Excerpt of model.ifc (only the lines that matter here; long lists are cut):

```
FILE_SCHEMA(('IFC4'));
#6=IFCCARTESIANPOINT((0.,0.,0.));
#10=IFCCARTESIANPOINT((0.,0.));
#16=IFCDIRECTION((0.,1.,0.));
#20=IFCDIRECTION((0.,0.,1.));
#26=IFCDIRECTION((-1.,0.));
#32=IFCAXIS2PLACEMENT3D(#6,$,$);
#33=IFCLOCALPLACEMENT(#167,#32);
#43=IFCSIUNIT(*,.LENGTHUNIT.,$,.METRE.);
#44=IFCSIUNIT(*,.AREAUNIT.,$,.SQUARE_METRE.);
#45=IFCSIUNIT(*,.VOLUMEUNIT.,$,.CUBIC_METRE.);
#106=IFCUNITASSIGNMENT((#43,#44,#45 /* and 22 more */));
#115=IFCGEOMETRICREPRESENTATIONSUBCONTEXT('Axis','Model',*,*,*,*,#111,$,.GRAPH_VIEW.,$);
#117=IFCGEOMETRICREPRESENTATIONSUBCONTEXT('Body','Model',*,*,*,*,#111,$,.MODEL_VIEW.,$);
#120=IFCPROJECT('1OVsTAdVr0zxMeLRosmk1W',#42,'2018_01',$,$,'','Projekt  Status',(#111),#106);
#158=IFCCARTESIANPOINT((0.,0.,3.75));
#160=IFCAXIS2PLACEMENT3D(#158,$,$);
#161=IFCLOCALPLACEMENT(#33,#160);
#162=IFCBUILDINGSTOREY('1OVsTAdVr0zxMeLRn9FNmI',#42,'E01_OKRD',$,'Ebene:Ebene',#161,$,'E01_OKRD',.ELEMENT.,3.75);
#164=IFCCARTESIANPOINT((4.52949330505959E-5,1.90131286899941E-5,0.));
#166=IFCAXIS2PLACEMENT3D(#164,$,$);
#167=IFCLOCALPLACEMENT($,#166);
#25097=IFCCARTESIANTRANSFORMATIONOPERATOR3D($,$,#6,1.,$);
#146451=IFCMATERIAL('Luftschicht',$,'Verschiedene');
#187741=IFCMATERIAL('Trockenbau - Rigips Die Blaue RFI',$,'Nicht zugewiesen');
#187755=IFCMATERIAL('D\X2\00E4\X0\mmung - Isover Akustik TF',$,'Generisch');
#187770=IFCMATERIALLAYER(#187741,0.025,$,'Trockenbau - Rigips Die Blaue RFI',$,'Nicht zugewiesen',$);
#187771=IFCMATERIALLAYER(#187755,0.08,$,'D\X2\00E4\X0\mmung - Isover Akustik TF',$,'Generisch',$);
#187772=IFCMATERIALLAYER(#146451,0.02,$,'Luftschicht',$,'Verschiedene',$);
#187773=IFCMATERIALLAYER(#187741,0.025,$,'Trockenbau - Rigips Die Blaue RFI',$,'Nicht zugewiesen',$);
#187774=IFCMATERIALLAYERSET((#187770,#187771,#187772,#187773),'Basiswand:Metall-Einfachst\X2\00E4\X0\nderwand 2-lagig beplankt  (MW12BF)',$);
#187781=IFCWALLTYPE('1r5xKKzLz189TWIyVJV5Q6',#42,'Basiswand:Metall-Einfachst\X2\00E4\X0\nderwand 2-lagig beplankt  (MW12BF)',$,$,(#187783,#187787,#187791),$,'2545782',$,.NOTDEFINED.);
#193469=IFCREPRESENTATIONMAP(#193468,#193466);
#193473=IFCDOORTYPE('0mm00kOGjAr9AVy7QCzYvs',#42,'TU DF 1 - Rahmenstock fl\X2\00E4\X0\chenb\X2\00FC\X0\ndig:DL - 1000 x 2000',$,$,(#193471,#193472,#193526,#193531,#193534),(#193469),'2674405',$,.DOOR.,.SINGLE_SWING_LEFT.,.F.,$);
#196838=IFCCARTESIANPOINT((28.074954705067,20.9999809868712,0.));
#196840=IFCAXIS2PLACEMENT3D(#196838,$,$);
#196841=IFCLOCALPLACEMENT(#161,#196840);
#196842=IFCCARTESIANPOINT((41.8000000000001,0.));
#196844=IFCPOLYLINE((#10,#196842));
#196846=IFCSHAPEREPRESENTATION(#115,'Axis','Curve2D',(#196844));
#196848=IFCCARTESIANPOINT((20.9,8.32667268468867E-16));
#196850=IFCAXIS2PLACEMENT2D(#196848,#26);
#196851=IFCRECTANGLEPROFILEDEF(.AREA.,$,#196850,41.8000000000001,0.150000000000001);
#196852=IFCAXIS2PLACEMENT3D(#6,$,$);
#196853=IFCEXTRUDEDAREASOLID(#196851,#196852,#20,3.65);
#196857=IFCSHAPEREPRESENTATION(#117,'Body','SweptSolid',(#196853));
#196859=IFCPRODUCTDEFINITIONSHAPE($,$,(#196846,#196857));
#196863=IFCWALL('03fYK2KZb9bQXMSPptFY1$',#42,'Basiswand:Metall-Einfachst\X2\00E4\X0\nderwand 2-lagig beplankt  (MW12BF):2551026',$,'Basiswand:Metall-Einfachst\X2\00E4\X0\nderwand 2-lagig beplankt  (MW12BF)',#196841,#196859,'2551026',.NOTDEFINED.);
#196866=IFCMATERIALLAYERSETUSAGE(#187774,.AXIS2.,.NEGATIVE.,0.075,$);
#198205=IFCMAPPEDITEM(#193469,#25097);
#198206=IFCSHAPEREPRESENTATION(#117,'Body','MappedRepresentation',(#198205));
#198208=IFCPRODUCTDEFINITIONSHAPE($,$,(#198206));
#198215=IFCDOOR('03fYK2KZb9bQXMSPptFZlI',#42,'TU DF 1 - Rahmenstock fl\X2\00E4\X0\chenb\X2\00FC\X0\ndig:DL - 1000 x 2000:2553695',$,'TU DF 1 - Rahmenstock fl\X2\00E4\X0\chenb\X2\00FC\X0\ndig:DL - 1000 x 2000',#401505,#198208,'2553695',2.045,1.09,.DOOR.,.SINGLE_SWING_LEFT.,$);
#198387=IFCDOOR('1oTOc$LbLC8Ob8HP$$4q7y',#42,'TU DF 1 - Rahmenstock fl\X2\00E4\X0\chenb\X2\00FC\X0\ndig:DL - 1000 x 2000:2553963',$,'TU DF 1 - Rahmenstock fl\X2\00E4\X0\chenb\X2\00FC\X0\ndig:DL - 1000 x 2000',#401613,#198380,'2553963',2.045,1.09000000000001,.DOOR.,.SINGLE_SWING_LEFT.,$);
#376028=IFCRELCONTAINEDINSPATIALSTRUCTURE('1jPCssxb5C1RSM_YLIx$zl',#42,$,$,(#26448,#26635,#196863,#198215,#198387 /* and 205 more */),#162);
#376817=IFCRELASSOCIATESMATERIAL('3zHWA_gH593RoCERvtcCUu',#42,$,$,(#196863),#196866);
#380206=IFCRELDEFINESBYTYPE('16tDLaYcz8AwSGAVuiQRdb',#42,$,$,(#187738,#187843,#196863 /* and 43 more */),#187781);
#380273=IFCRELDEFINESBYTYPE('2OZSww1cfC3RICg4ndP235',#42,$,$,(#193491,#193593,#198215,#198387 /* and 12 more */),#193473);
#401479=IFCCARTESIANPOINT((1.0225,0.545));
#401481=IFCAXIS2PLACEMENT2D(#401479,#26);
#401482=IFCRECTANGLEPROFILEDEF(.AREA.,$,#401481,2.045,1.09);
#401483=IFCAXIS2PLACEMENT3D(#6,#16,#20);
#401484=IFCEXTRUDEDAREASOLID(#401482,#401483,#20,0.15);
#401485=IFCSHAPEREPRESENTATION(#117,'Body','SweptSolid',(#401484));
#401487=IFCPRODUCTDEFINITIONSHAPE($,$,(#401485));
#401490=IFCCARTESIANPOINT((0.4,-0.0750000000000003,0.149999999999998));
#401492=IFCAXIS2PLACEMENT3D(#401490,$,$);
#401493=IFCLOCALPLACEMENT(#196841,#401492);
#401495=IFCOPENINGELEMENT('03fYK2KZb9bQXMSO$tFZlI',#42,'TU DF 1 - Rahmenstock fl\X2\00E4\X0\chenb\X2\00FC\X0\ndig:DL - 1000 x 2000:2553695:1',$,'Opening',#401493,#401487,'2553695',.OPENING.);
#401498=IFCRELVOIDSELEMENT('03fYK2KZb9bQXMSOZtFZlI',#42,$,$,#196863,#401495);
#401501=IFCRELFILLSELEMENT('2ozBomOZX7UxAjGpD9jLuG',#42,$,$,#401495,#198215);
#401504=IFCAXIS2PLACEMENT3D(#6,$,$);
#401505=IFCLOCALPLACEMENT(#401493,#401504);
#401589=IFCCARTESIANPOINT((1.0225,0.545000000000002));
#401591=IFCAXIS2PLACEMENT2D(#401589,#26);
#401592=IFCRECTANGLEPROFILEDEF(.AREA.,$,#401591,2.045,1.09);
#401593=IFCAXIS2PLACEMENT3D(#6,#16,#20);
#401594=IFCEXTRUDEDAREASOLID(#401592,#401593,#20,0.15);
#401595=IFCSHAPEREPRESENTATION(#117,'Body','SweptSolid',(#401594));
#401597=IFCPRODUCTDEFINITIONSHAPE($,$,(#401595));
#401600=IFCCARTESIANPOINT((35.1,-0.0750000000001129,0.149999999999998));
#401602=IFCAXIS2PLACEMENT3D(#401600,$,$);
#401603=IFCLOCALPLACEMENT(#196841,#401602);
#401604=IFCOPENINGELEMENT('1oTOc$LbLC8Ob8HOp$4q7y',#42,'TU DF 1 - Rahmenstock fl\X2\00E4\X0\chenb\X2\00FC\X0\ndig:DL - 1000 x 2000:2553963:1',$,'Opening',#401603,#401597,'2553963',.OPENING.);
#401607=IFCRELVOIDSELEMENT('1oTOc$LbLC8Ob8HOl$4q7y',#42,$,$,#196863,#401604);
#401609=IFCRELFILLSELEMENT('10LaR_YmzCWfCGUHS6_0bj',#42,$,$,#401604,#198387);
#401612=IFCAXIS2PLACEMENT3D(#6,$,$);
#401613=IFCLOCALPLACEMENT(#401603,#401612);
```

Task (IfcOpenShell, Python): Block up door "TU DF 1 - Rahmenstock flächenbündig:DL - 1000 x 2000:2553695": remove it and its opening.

```python
import ifcopenshell
import ifcopenshell.api.feature
import ifcopenshell.api.root
import ifcopenshell.geom
import ifcopenshell.util.shape

model = ifcopenshell.open("model.ifc")
settings = ifcopenshell.geom.settings()


def volume(element):
    """Net volume in cubic metres, openings subtracted."""
    shape = ifcopenshell.geom.create_shape(settings, element)
    return ifcopenshell.util.shape.get_volume(shape.geometry)


door = model.by_id(198215)
opening = door.FillsVoids[0].RelatingOpeningElement
wall = opening.VoidsElements[0].RelatingBuildingElement
before = volume(wall)

ifcopenshell.api.root.remove_product(model, product=door)
ifcopenshell.api.feature.remove_feature(model, feature=opening)

after = volume(wall)

print(f"wall volume {before:.3f} -> {after:.3f} m3")

model.write("model_v2.ifc")
```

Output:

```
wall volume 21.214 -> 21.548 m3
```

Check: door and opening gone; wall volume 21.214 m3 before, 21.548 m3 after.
